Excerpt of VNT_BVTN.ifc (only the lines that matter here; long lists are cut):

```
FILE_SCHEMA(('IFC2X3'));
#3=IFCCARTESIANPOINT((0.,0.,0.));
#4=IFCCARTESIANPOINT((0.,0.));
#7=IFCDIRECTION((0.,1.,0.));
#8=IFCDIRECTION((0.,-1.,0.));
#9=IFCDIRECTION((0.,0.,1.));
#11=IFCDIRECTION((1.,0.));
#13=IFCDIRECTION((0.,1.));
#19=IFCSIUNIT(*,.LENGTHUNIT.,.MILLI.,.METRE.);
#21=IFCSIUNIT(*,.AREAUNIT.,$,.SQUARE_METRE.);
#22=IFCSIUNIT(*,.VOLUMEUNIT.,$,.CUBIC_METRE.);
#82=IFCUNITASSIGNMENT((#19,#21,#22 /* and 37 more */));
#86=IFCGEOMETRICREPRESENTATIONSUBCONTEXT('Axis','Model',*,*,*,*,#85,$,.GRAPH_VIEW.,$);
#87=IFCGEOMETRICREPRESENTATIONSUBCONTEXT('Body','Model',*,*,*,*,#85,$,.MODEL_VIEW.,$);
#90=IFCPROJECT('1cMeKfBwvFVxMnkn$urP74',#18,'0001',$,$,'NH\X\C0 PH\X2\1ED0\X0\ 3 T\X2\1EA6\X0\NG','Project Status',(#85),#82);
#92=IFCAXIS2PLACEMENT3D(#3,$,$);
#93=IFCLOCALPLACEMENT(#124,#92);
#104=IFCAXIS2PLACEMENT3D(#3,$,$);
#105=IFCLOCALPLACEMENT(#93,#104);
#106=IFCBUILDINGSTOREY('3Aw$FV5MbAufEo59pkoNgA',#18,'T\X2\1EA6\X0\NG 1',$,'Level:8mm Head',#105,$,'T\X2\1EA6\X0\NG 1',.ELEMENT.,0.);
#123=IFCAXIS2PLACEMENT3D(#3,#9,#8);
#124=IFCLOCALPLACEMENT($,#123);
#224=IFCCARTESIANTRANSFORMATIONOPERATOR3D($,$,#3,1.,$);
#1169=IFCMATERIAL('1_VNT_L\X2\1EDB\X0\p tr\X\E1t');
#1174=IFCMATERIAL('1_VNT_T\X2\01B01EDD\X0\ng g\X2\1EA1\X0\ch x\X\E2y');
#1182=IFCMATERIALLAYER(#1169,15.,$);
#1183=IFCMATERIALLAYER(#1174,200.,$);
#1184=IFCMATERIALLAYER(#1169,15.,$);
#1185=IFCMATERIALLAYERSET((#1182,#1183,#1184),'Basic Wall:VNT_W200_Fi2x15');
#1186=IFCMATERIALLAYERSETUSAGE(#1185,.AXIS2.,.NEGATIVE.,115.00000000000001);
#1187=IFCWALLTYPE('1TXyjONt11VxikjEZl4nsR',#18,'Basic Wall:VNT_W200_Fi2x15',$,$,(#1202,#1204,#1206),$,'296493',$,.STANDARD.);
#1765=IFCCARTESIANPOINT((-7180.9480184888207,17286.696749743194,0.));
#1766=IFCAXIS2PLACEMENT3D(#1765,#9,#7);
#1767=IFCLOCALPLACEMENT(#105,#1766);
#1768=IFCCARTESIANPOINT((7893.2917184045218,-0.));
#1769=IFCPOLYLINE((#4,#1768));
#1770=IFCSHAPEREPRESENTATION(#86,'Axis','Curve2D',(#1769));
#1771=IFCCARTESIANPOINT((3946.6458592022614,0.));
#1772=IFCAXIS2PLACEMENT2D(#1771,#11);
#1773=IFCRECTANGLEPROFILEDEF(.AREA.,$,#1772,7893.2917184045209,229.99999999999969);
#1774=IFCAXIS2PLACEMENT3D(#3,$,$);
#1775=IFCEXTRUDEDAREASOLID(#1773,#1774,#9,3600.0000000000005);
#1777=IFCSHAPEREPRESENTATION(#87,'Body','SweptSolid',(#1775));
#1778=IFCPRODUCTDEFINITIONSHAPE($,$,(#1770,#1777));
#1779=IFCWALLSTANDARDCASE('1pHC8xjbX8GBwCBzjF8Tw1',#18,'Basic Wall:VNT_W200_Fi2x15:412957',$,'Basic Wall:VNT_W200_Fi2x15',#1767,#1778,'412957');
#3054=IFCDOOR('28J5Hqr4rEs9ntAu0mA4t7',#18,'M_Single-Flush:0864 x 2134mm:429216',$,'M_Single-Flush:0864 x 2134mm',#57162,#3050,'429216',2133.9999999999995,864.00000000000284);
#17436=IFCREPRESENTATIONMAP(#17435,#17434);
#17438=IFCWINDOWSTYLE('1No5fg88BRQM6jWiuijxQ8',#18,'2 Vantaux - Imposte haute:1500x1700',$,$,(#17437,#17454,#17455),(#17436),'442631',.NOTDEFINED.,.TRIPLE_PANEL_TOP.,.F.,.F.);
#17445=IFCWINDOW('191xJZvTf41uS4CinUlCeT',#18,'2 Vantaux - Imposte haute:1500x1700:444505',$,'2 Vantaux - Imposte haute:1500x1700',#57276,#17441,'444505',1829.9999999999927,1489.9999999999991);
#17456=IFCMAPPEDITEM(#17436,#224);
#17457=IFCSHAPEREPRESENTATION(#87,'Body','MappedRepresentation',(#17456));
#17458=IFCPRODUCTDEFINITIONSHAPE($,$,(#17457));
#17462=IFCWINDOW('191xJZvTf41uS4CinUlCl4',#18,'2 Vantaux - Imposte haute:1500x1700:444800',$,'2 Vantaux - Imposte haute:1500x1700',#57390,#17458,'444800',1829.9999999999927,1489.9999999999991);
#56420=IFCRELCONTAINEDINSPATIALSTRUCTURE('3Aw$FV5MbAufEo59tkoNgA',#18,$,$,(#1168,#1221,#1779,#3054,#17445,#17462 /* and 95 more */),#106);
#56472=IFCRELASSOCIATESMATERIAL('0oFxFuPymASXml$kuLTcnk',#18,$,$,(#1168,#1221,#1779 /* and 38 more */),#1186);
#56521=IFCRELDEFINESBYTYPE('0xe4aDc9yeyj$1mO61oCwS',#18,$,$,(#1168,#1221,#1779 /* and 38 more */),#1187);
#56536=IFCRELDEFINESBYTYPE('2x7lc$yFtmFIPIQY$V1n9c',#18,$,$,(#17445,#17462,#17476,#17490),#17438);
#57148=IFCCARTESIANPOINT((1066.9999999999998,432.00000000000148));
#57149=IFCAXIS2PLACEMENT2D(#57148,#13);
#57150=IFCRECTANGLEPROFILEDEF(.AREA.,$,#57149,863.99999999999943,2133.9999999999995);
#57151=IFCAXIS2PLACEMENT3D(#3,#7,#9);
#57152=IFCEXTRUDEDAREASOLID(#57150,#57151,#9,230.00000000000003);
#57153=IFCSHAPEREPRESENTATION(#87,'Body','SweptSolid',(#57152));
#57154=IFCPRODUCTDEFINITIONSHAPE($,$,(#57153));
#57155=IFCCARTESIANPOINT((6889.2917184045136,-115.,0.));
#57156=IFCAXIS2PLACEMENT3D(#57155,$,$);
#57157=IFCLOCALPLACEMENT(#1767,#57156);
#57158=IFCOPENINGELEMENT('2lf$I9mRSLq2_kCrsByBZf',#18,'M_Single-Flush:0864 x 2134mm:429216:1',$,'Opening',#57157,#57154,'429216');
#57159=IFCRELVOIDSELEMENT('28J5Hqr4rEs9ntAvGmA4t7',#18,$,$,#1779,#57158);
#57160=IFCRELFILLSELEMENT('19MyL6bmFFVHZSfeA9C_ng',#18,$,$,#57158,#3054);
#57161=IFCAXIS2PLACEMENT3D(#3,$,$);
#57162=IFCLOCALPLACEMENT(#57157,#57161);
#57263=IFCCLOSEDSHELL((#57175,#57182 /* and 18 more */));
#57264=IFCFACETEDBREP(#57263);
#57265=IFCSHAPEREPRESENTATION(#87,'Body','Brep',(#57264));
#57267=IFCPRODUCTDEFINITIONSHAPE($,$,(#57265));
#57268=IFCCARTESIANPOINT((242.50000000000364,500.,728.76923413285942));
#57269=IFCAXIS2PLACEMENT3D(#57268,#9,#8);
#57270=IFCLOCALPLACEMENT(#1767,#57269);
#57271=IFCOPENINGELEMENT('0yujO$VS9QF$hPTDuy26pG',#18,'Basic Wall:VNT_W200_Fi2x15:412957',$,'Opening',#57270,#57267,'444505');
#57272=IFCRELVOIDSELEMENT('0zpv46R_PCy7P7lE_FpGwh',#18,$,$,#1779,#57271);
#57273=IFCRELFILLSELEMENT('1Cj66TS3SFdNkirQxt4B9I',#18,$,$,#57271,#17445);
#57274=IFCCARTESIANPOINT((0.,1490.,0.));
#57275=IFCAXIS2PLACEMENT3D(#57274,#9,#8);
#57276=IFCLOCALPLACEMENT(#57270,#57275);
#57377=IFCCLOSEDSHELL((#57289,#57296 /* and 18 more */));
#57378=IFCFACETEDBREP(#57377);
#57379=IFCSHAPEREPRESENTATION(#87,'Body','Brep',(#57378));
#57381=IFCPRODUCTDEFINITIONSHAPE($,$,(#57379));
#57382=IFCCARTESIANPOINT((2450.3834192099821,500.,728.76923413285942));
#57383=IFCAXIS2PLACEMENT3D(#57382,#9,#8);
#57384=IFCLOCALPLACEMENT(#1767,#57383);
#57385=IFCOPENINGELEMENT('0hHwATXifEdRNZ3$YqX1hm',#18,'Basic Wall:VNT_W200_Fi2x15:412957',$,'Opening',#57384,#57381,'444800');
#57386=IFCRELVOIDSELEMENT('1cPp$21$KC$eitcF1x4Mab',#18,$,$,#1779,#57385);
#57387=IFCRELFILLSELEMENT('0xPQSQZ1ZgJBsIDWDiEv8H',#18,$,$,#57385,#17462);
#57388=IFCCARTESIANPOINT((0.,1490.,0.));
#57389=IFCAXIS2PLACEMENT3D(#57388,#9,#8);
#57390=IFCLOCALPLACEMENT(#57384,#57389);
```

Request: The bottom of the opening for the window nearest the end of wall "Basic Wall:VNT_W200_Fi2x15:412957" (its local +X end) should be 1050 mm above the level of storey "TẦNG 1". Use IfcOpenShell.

```python
import numpy as np
import ifcopenshell
import ifcopenshell.api.geometry
import ifcopenshell.geom
import ifcopenshell.util.element
import ifcopenshell.util.placement
import ifcopenshell.util.shape
import ifcopenshell.util.unit

model = ifcopenshell.open("VNT_BVTN.ifc")
unit_scale = ifcopenshell.util.unit.calculate_unit_scale(model)

window = model.by_guid("191xJZvTf41uS4CinUlCl4")
opening = window.FillsVoids[0].RelatingOpeningElement
storey = ifcopenshell.util.element.get_container(window, ifc_class="IfcBuildingStorey")
level = ifcopenshell.util.placement.get_local_placement(storey.ObjectPlacement)[2, 3]

# The opening's origin need not be at the sill, so measure its lowest point.
shape = ifcopenshell.geom.create_shape(ifcopenshell.geom.settings(), opening)
bottom = ifcopenshell.util.shape.get_shape_bottom_elevation(shape, shape.geometry) / unit_scale
dz = level + 1.05 / unit_scale - bottom

shift = np.array([0.0, 0.0, dz])
# The window is placed relative to its opening, so it follows when the opening moves.
matrix = ifcopenshell.util.placement.get_local_placement(opening.ObjectPlacement)
matrix[:3, 3] += shift
ifcopenshell.api.geometry.edit_object_placement(
    model, product=opening, matrix=matrix, is_si=False, should_transform_children=True
)

print(f"moved by {dz * unit_scale:+.3f} m")

model.write("VNT_BVTN_rev.ifc")
```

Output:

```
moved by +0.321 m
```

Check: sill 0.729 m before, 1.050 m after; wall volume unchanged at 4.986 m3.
